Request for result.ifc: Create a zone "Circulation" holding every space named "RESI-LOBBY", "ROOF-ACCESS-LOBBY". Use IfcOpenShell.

First a look at what the model holds.

```python
import ifcopenshell

model = ifcopenshell.open("result.ifc")
print(model.schema)
seen = {}
for space in model.by_type("IfcSpace"):
    seen[space.Name] = seen.get(space.Name, 0) + 1
for name, count in sorted(seen.items(), key=str):
    print(count, "x", name)
print("zones:", [z.Name for z in model.by_type("IfcZone")][:20])
```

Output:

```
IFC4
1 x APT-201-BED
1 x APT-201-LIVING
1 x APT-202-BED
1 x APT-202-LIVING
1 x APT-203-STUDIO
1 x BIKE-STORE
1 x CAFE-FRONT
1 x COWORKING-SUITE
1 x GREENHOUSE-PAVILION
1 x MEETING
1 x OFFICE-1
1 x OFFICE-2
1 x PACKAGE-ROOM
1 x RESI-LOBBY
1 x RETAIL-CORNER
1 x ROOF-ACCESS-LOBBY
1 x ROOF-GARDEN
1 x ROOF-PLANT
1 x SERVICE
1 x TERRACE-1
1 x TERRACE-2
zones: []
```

```python
import ifcopenshell
import ifcopenshell.api.group
import ifcopenshell.api.root

model = ifcopenshell.open("result.ifc")

names = {"RESI-LOBBY", "ROOF-ACCESS-LOBBY"}
spaces = [s for s in model.by_type("IfcSpace") if s.Name in names]

zone = ifcopenshell.api.root.create_entity(model, ifc_class="IfcZone", name="Circulation")
ifcopenshell.api.group.assign_group(model, products=spaces, group=zone)
print(len(spaces), "spaces in", zone.Name)

model.write("result_v2.ifc")
```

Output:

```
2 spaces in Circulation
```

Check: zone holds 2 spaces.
